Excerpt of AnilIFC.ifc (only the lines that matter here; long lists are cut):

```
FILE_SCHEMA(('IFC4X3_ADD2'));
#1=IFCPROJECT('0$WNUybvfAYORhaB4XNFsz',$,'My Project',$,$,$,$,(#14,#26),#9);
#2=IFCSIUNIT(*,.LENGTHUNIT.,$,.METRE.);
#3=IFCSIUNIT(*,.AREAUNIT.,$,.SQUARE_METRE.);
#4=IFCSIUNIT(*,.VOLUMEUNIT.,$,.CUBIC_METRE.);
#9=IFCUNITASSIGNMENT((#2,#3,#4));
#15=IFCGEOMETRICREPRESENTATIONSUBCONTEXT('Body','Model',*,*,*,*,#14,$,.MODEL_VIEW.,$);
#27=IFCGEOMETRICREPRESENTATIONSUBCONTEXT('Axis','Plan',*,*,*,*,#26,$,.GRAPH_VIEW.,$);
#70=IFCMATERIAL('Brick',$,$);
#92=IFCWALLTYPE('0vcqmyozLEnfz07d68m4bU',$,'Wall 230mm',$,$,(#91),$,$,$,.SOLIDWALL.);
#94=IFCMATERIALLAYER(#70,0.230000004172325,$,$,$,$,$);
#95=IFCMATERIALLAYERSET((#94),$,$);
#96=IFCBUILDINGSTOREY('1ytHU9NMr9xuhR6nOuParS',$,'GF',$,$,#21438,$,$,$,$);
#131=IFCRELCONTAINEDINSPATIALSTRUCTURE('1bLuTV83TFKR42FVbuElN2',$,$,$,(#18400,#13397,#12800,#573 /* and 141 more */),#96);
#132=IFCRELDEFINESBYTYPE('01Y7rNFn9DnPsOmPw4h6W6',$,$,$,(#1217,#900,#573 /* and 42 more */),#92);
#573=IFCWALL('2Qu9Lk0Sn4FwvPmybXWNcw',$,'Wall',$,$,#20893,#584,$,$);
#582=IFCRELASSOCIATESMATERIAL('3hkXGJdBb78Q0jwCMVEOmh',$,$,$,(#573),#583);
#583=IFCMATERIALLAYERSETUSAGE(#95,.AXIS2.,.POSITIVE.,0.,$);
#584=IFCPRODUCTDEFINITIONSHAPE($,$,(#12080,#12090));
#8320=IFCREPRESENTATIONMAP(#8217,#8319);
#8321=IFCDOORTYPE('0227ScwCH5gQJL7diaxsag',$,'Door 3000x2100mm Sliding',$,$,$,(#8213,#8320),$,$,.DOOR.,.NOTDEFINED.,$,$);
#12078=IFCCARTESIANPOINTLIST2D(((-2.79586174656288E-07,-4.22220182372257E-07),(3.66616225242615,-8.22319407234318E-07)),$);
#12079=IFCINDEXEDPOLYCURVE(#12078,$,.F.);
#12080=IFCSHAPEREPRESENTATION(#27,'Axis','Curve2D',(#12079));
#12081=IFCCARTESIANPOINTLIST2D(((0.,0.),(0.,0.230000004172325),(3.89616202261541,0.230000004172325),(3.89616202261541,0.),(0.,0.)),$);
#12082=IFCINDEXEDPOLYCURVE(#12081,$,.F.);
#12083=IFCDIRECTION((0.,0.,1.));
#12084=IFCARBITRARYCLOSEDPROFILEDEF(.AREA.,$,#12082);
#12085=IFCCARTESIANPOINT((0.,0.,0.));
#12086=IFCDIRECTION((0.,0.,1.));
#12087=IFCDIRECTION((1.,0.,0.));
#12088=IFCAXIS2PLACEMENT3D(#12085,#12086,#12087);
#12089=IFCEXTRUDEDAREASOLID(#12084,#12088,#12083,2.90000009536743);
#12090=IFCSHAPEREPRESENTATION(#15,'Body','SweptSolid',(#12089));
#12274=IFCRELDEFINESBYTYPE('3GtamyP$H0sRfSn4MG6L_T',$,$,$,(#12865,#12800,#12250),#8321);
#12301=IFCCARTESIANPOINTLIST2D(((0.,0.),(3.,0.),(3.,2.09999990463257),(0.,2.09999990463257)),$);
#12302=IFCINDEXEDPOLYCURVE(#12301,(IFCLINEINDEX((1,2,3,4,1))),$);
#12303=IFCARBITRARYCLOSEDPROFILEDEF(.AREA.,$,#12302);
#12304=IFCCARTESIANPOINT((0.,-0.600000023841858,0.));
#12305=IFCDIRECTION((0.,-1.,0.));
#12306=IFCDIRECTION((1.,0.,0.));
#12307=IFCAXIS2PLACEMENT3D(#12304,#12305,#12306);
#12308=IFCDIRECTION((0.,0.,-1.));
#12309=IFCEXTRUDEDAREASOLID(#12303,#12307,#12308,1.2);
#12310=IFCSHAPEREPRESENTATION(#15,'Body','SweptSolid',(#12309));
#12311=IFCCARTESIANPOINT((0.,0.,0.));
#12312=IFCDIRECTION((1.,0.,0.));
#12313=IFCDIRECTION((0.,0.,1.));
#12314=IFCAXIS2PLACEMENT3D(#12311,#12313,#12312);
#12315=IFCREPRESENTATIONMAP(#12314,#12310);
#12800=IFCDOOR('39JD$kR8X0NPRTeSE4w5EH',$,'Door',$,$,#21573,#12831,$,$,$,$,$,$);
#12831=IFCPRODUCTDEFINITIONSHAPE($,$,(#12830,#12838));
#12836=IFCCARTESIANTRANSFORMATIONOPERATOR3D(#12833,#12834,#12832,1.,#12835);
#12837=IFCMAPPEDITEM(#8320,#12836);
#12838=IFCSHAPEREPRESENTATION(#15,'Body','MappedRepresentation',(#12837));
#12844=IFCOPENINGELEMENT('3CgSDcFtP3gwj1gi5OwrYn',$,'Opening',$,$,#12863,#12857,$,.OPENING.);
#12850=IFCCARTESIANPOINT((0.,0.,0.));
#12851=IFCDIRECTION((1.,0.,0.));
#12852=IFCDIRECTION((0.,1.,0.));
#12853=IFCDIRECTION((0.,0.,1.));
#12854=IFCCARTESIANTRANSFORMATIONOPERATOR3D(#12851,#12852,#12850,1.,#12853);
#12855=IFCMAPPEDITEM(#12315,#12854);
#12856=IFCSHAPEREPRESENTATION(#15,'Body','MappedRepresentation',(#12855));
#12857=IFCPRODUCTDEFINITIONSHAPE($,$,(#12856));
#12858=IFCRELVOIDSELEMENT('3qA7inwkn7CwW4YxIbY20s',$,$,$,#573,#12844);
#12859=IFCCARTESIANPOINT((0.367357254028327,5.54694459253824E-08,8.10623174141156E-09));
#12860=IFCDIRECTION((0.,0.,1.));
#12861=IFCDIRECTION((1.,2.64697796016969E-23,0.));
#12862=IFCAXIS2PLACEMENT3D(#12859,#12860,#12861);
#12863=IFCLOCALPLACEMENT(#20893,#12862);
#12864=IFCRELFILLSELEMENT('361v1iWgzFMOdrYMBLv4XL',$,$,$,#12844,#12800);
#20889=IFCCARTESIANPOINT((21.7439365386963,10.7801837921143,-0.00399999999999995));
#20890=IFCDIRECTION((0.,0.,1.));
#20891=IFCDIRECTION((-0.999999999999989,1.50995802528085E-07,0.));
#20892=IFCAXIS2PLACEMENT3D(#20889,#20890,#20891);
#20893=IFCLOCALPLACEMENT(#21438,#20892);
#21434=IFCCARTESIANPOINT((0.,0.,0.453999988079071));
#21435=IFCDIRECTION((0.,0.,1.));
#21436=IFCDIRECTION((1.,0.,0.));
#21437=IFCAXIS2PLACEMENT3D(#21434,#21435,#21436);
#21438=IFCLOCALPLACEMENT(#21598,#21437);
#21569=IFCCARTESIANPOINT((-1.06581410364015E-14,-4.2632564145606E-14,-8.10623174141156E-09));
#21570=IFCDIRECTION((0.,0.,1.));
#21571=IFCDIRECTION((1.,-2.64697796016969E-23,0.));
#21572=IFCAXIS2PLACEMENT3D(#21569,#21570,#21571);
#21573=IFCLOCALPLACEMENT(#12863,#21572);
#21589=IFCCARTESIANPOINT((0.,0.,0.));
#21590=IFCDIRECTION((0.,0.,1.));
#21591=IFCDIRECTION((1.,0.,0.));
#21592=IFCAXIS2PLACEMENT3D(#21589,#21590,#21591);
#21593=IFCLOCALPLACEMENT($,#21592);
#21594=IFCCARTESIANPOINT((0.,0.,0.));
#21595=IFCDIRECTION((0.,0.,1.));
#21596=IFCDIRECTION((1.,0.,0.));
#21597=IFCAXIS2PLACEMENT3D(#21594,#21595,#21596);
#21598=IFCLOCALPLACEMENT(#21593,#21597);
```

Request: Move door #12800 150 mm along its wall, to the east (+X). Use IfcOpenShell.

```python
import ifcopenshell
import ifcopenshell.api.geometry
import ifcopenshell.util.placement
import ifcopenshell.util.unit

model = ifcopenshell.open("AnilIFC.ifc")
unit_scale = ifcopenshell.util.unit.calculate_unit_scale(model)

door = model.by_guid("39JD$kR8X0NPRTeSE4w5EH")
opening = door.FillsVoids[0].RelatingOpeningElement
wall = opening.VoidsElements[0].RelatingBuildingElement

wall_matrix = ifcopenshell.util.placement.get_local_placement(wall.ObjectPlacement)
shift = wall_matrix[:3, 0] * -0.15 / unit_scale
before = ifcopenshell.util.placement.get_local_placement(door.ObjectPlacement)[:3, 3].copy()

# The door is placed relative to its opening, so it follows when the opening moves.
matrix = ifcopenshell.util.placement.get_local_placement(opening.ObjectPlacement)
matrix[:3, 3] += shift
ifcopenshell.api.geometry.edit_object_placement(
    model, product=opening, matrix=matrix, is_si=False, should_transform_children=True
)

after = ifcopenshell.util.placement.get_local_placement(door.ObjectPlacement)[:3, 3]
print("door moved by", (after - before).round(3) + 0.0)

model.write("AnilIFC_v2.ifc")
```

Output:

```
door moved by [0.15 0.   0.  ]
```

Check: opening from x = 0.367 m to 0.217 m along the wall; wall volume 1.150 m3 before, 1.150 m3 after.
